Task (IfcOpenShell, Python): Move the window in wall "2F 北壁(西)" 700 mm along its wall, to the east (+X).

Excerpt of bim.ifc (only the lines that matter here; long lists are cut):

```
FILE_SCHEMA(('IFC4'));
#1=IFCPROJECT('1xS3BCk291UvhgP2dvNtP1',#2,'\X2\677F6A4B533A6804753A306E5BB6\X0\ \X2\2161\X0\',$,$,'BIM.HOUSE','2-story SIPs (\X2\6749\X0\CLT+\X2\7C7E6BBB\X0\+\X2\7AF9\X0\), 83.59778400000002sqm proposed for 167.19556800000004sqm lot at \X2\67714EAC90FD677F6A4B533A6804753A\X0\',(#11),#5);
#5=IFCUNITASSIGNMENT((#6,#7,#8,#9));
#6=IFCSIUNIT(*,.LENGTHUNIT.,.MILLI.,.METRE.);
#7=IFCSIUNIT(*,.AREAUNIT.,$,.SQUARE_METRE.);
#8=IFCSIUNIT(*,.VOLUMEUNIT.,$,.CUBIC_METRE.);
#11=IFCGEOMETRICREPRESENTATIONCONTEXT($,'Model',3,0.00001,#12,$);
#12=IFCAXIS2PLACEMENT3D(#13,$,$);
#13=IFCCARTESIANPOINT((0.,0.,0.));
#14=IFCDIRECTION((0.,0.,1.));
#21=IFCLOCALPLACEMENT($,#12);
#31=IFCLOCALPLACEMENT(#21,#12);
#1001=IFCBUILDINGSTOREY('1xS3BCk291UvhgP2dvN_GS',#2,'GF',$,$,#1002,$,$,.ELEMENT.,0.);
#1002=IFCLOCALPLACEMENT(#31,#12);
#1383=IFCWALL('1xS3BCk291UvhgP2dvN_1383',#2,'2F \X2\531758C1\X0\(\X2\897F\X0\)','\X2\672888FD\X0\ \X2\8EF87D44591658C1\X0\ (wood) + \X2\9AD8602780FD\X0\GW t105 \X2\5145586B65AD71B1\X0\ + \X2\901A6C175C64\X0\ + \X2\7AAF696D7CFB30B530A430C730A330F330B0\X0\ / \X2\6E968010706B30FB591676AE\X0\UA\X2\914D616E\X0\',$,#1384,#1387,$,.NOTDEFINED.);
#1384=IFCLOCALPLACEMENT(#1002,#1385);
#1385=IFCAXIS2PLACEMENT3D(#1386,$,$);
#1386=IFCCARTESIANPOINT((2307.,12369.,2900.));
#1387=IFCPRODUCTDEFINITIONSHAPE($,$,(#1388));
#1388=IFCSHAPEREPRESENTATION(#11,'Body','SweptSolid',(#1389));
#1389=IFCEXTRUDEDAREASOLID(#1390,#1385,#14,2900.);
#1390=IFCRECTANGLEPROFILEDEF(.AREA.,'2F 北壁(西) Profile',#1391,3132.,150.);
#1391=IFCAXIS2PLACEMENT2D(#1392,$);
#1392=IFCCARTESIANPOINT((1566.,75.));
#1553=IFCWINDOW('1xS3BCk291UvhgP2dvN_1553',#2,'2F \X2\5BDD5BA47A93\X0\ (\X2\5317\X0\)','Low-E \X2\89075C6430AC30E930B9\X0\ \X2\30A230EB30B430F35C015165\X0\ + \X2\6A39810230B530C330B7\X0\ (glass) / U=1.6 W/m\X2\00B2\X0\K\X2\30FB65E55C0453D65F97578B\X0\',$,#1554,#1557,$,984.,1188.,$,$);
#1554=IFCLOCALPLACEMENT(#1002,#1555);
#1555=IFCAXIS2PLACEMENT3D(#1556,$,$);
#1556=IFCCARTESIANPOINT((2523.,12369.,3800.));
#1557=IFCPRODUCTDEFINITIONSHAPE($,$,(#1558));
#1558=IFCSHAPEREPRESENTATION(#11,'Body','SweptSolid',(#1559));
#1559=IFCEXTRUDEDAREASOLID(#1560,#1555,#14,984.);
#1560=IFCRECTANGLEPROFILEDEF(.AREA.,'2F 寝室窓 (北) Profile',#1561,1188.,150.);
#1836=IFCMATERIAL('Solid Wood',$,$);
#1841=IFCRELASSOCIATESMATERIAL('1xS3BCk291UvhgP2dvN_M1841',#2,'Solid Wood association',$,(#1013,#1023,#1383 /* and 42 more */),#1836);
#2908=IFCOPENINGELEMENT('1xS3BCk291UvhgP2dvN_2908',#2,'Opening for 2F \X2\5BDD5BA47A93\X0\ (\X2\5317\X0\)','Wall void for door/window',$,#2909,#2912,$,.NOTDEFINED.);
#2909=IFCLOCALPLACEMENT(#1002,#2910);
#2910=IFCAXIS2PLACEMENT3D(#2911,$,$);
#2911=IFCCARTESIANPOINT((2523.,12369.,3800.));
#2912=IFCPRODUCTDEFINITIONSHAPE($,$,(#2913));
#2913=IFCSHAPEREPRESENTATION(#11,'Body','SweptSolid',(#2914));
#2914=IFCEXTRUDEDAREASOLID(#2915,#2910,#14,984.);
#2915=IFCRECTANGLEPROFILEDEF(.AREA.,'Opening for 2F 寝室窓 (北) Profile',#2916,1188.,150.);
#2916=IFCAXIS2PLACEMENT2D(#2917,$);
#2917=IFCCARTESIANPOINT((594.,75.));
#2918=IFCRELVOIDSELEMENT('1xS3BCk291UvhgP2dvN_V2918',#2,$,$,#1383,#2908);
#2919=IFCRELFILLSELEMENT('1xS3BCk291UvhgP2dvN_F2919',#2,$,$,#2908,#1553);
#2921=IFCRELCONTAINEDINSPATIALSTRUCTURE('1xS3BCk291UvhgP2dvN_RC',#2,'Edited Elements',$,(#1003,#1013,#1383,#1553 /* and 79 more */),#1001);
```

```python
import ifcopenshell
import ifcopenshell.api.geometry
import ifcopenshell.util.placement
import ifcopenshell.util.unit

model = ifcopenshell.open("bim.ifc")
unit_scale = ifcopenshell.util.unit.calculate_unit_scale(model)

window = model.by_id(1553)
opening = window.FillsVoids[0].RelatingOpeningElement
wall = opening.VoidsElements[0].RelatingBuildingElement

wall_matrix = ifcopenshell.util.placement.get_local_placement(wall.ObjectPlacement)
shift = wall_matrix[:3, 0] * 0.7 / unit_scale
before = ifcopenshell.util.placement.get_local_placement(window.ObjectPlacement)[:3, 3].copy()

# The window is not placed relative to its opening, so move both.
for product in (opening, window):
    matrix = ifcopenshell.util.placement.get_local_placement(product.ObjectPlacement)
    matrix[:3, 3] += shift
    ifcopenshell.api.geometry.edit_object_placement(model, product=product, matrix=matrix, is_si=False)

after = ifcopenshell.util.placement.get_local_placement(window.ObjectPlacement)[:3, 3]
print("window moved by", (after - before).round(3) + 0.0)

model.write("bim_edited.ifc")
```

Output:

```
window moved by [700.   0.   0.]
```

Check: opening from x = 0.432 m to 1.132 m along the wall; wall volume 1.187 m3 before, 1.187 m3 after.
